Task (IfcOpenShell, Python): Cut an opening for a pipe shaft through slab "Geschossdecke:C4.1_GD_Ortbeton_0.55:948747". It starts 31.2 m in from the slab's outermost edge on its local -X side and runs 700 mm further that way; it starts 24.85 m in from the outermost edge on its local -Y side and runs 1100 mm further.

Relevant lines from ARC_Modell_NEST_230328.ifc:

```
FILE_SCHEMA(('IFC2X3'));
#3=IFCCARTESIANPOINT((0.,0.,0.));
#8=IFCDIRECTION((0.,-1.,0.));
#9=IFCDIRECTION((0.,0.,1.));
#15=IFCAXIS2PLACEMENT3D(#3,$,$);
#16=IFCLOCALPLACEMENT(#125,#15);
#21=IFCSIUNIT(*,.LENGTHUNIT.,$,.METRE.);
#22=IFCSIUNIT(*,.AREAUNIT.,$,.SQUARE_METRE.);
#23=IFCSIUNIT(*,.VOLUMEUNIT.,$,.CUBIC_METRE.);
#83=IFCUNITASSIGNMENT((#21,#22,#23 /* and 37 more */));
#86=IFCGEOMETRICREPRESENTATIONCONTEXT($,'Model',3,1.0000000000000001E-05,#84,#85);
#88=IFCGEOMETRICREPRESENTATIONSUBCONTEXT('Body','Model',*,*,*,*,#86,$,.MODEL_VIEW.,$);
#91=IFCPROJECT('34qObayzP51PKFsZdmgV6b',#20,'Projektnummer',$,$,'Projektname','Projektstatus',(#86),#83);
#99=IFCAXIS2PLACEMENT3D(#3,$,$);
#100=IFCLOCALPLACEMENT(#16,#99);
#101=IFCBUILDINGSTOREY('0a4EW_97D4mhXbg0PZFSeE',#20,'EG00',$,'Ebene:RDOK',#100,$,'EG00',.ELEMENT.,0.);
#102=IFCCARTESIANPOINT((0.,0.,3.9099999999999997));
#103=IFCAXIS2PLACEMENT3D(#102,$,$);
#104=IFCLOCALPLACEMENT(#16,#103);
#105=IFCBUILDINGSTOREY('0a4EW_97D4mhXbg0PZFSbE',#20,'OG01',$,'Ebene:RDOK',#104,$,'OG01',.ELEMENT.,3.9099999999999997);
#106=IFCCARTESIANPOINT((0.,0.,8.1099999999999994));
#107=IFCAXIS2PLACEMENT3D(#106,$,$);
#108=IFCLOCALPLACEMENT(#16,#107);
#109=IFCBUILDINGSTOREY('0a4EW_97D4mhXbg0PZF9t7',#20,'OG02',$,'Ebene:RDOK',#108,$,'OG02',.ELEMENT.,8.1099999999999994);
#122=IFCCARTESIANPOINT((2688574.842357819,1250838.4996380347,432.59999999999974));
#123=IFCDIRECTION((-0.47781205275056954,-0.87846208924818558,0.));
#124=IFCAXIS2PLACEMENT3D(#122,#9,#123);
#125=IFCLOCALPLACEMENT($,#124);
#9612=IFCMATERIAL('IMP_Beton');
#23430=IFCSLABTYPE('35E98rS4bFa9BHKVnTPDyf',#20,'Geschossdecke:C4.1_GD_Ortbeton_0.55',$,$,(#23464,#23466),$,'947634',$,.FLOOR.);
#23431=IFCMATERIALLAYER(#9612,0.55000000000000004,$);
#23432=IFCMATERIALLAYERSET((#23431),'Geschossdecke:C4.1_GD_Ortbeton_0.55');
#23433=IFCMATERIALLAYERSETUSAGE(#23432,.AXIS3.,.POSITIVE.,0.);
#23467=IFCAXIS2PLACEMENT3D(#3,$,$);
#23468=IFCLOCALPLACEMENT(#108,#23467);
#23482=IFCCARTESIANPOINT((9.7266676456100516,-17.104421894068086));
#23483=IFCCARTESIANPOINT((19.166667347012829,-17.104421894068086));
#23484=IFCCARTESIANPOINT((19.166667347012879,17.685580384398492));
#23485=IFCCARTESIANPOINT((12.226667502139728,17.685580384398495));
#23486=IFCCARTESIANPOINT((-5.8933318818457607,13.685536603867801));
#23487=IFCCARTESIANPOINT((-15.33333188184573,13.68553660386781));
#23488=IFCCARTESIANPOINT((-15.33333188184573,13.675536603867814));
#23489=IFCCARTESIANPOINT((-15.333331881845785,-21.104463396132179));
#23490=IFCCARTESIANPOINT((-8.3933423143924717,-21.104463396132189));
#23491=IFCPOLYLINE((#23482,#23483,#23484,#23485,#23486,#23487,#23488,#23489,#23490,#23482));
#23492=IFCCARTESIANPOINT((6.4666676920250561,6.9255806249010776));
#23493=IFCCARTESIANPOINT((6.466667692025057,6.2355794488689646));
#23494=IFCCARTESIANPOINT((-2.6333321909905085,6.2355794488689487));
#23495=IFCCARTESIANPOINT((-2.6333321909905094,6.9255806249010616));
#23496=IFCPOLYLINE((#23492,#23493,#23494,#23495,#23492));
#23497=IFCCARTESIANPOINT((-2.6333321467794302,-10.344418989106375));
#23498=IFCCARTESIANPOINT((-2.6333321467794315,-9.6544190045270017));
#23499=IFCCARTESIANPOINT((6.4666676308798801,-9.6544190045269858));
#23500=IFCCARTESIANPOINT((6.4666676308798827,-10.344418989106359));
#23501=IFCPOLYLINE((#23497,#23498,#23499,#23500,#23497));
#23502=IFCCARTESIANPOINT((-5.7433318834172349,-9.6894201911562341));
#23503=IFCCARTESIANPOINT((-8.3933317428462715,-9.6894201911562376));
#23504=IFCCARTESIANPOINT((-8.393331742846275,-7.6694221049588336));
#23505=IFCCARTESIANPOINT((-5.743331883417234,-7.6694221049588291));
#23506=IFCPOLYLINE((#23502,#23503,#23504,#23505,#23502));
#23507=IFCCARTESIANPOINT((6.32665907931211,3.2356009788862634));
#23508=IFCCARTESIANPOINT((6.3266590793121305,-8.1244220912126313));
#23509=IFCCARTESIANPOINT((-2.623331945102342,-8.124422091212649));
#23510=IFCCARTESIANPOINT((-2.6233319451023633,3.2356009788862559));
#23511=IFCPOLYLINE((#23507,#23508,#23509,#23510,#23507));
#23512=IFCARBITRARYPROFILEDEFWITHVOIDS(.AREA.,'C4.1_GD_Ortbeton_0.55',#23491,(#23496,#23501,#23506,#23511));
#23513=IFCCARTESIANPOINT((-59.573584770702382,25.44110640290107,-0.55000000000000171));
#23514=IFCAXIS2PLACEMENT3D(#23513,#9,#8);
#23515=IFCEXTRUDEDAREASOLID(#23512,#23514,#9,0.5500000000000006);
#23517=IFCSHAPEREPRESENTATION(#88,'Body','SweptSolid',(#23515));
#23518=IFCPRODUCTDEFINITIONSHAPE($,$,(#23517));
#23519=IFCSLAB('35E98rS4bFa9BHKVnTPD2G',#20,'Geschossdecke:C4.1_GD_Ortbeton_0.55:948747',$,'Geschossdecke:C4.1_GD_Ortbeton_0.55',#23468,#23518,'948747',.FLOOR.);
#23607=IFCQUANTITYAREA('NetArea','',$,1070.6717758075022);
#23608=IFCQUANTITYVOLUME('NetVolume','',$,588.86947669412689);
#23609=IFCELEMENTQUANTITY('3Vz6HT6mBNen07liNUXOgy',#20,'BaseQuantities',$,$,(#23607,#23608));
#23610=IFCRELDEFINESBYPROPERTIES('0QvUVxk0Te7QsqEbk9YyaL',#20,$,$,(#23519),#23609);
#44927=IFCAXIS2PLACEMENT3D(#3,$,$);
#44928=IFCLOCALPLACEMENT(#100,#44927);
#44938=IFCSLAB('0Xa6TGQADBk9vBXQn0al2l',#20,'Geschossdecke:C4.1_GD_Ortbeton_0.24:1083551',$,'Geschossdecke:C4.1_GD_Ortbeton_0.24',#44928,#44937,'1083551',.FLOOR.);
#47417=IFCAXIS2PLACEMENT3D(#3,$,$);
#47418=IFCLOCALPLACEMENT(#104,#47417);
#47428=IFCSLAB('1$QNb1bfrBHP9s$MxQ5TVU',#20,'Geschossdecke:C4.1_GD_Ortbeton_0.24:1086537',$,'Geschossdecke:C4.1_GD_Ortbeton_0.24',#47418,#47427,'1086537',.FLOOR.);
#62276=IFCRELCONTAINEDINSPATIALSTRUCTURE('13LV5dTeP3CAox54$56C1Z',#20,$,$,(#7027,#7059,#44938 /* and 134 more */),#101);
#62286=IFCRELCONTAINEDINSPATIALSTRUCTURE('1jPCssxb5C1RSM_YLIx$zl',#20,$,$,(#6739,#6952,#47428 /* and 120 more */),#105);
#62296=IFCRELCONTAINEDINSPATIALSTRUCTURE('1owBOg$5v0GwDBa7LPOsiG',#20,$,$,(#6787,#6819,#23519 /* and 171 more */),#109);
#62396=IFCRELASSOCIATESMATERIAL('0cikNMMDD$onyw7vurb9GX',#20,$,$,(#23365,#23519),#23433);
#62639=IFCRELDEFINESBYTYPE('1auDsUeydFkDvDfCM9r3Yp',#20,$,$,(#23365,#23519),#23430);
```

```python
import numpy as np
import ifcopenshell
import ifcopenshell.api.feature
import ifcopenshell.api.geometry
import ifcopenshell.api.pset
import ifcopenshell.api.root
import ifcopenshell.geom
import ifcopenshell.util.element
import ifcopenshell.util.placement
import ifcopenshell.util.representation
import ifcopenshell.util.shape
import ifcopenshell.util.unit

model = ifcopenshell.open("ARC_Modell_NEST_230328.ifc")
unit_scale = ifcopenshell.util.unit.calculate_unit_scale(model)
area_scale = ifcopenshell.util.unit.calculate_unit_scale(model, "AREAUNIT")
volume_scale = ifcopenshell.util.unit.calculate_unit_scale(model, "VOLUMEUNIT")
settings = ifcopenshell.geom.settings()


def volume(element):
    """Net volume in cubic metres, openings subtracted."""
    shape = ifcopenshell.geom.create_shape(settings, element)
    return ifcopenshell.util.shape.get_volume(shape.geometry)


slab = model.by_guid("35E98rS4bFa9BHKVnTPD2G")
before = volume(slab)

# Extent in the slab's own axes, in metres. The edges named are its -X and -Y sides.
slab_shape = ifcopenshell.geom.create_shape(settings, slab)
vertices = ifcopenshell.util.shape.get_vertices(slab_shape.geometry)
x_min, y_min, bottom = vertices.min(axis=0)
top = vertices[:, 2].max()

opening = ifcopenshell.api.root.create_entity(model, ifc_class="IfcOpeningElement", name="Pipe shaft opening")
context = ifcopenshell.util.representation.get_context(model, "Model", "Body", "MODEL_VIEW")
width, depth = 0.7, 1.1
outline = [(0.0, 0.0), (width, 0.0), (width, depth), (0.0, depth), (0.0, 0.0)]
# Overshoot both faces by 50 mm so the cut is clean.
shape = ifcopenshell.api.geometry.add_slab_representation(
    model, context=context, depth=top - bottom + 0.1, polyline=outline
)
ifcopenshell.api.geometry.assign_representation(model, product=opening, representation=shape)

matrix = ifcopenshell.util.placement.get_local_placement(slab.ObjectPlacement)
matrix[:, 3] = matrix @ np.append(np.array([x_min + 31.2, y_min + 24.85, bottom - 0.05]) / unit_scale, 1.0)
ifcopenshell.api.geometry.edit_object_placement(model, product=opening, matrix=matrix, is_si=False)
ifcopenshell.api.feature.add_feature(model, feature=opening, element=slab)

after = volume(slab)

# Update the slab's stored quantities.
qto = model.by_id(ifcopenshell.util.element.get_pset(slab, "BaseQuantities", should_inherit=False)["id"])
ifcopenshell.api.pset.edit_qto(model, qto=qto, properties={
    "NetArea": after / (top - bottom) / area_scale,
    "NetVolume": after / volume_scale,
})

print(f"slab volume {before:.3f} -> {after:.3f} m3")

model.write("ARC_Modell_NEST_230328_rev.ifc")
```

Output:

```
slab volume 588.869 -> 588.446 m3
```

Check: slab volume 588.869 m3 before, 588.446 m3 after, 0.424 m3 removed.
